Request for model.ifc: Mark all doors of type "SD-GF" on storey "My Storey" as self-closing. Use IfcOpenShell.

First a look at what the model holds.

```python
import ifcopenshell
import ifcopenshell.util.element

model = ifcopenshell.open("model.ifc")
print(model.schema)
storey = next(s for s in model.by_type("IfcBuildingStorey") if s.Name == "My Storey")
doors = [e for e in ifcopenshell.util.element.get_decomposition(storey) if e.is_a("IfcDoor")]
seen = {}
for e in doors:
    element_type = ifcopenshell.util.element.get_type(e)
    key = (element_type.Name if element_type != e and element_type else None, ifcopenshell.util.element.get_pset(e, "Pset_DoorCommon", "SelfClosing"))
    seen[key] = seen.get(key, 0) + 1
for (name, value), count in sorted(seen.items(), key=str):
    print(count, "x", name, "|", value)
```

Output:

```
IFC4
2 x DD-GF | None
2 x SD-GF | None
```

```python
import ifcopenshell
import ifcopenshell.api.pset
import ifcopenshell.util.element

model = ifcopenshell.open("model.ifc")

storey = next(s for s in model.by_type("IfcBuildingStorey") if s.Name == "My Storey")
doors = [e for e in ifcopenshell.util.element.get_decomposition(storey) if e.is_a("IfcDoor")]

count = 0
for e in doors:
    element_type = ifcopenshell.util.element.get_type(e)
    if element_type in (None, e) or element_type.Name != "SD-GF":
        continue
    # add_pset returns the element's existing set when there is one.
    pset = ifcopenshell.api.pset.add_pset(model, product=e, name="Pset_DoorCommon")
    ifcopenshell.api.pset.edit_pset(model, pset=pset, properties={"SelfClosing": True})
    count += 1

print(count, "doors updated")

model.write("model_updated.ifc")
```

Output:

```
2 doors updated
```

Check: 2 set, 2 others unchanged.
